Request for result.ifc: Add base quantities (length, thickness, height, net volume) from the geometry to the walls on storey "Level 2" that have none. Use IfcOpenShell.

First a look at what the model holds.

```python
import ifcopenshell
import ifcopenshell.util.element
import ifcopenshell.util.unit

model = ifcopenshell.open("result.ifc")
print(model.schema)
for unit_type in ("LENGTHUNIT", "AREAUNIT", "VOLUMEUNIT"):
    print(unit_type, ifcopenshell.util.unit.calculate_unit_scale(model, unit_type))
storey = next(s for s in model.by_type("IfcBuildingStorey") if s.Name == "Level 2")
walls = [e for e in ifcopenshell.util.element.get_decomposition(storey) if e.is_a("IfcWall")]
for e in sorted(walls, key=lambda e: e.id()):
    print(e.id(), e.is_a(), e.Name, list(ifcopenshell.util.element.get_psets(e, qtos_only=True)), sep=" | ")
```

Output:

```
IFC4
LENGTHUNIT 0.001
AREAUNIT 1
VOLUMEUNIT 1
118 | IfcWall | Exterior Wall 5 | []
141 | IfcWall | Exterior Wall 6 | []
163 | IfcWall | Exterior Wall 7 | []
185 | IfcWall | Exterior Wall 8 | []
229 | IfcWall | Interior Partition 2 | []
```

```python
import ifcopenshell
import ifcopenshell.api.pset
import ifcopenshell.geom
import ifcopenshell.util.element
import ifcopenshell.util.shape
import ifcopenshell.util.unit

model = ifcopenshell.open("result.ifc")
unit_scale = ifcopenshell.util.unit.calculate_unit_scale(model)
volume_scale = ifcopenshell.util.unit.calculate_unit_scale(model, "VOLUMEUNIT")
settings = ifcopenshell.geom.settings()

storey = next(s for s in model.by_type("IfcBuildingStorey") if s.Name == "Level 2")
walls = [e for e in ifcopenshell.util.element.get_decomposition(storey) if e.is_a("IfcWall")]

for e in sorted(walls, key=lambda e: e.id()):
    if ifcopenshell.util.element.get_psets(e, qtos_only=True, should_inherit=False):
        continue
    # Geometry comes back in metres, in the element's own axes.
    shape = ifcopenshell.geom.create_shape(settings, e)
    values = {
        "Length": ifcopenshell.util.shape.get_x(shape.geometry) / unit_scale,
        "Width": ifcopenshell.util.shape.get_y(shape.geometry) / unit_scale,
        "Height": ifcopenshell.util.shape.get_z(shape.geometry) / unit_scale,
        "NetVolume": ifcopenshell.util.shape.get_volume(shape.geometry) / volume_scale,
    }
    qto = ifcopenshell.api.pset.add_qto(model, product=e, name="Qto_WallBaseQuantities")
    ifcopenshell.api.pset.edit_qto(model, qto=qto, properties=values)
    print(e.id(), {k: round(v, 3) for k, v in values.items()})

model.write("result_edited.ifc")
```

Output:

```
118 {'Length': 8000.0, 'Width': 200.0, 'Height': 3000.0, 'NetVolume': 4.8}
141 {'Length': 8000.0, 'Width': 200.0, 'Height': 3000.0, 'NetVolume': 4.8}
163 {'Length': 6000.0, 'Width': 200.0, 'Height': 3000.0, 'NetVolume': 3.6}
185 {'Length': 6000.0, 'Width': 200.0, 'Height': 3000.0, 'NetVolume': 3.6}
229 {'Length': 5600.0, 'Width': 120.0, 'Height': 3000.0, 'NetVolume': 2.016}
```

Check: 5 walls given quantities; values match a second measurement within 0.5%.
